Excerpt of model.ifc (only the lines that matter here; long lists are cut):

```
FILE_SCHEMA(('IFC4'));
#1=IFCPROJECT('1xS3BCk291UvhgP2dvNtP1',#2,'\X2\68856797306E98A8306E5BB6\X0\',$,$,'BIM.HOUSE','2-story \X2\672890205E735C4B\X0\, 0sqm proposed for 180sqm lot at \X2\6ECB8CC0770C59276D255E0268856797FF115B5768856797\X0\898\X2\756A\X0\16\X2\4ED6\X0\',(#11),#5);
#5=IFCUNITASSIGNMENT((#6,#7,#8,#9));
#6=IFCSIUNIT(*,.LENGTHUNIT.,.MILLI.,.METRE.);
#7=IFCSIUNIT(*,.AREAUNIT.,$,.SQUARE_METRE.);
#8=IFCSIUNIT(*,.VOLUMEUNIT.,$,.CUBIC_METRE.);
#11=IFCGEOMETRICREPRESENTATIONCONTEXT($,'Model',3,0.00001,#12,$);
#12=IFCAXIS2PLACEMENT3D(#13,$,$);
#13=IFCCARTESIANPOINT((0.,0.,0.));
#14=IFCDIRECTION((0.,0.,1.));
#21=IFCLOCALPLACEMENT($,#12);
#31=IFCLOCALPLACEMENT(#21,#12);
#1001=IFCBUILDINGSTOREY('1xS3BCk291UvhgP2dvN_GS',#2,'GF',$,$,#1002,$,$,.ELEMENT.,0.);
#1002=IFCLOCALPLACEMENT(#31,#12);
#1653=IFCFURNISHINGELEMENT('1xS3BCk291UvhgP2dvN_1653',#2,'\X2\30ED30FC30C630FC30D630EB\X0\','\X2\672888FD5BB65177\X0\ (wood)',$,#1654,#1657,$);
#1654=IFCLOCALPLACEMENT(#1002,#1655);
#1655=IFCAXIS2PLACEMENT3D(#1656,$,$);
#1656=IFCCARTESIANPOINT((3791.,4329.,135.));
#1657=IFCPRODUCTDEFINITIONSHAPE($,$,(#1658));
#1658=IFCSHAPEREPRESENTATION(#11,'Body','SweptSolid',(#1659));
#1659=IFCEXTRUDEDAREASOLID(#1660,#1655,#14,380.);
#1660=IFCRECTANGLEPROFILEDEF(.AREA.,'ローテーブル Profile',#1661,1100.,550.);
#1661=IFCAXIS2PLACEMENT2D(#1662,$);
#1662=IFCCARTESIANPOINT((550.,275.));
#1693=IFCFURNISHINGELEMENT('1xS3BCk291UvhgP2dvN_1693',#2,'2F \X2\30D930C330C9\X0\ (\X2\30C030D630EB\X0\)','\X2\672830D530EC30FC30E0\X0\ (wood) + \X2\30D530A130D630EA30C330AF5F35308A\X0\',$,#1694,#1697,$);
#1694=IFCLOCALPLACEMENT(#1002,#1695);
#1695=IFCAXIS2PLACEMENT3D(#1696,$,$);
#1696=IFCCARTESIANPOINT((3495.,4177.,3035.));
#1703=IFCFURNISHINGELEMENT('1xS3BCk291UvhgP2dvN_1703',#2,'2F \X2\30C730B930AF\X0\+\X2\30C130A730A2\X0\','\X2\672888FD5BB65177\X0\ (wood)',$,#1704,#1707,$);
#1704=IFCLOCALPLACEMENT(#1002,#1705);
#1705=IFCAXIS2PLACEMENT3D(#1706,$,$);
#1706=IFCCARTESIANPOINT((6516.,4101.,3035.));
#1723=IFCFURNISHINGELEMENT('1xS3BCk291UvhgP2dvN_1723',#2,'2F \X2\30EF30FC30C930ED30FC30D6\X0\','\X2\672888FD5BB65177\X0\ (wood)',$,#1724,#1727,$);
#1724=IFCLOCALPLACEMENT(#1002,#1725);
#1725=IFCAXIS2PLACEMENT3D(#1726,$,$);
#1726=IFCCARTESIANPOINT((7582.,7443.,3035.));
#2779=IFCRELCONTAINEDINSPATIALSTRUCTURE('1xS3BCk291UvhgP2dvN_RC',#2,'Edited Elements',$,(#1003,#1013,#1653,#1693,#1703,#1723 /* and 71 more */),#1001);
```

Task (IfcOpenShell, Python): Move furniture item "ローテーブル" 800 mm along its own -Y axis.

```python
import ifcopenshell
import ifcopenshell.api.geometry
import ifcopenshell.util.placement
import ifcopenshell.util.unit

model = ifcopenshell.open("model.ifc")
unit_scale = ifcopenshell.util.unit.calculate_unit_scale(model)

item = model.by_guid("1xS3BCk291UvhgP2dvN_1653")
matrix = ifcopenshell.util.placement.get_local_placement(item.ObjectPlacement)
matrix[:3, 3] -= matrix[:3, 1] * 0.8 / unit_scale
ifcopenshell.api.geometry.edit_object_placement(model, product=item, matrix=matrix, is_si=False)

print(ifcopenshell.util.placement.get_local_placement(item.ObjectPlacement).round(3) + 0.0)

model.write("model_rev.ifc")
```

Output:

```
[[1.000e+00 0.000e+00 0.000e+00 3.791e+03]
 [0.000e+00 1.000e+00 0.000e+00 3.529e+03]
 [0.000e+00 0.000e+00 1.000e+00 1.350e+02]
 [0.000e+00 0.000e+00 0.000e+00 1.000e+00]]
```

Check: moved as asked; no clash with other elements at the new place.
